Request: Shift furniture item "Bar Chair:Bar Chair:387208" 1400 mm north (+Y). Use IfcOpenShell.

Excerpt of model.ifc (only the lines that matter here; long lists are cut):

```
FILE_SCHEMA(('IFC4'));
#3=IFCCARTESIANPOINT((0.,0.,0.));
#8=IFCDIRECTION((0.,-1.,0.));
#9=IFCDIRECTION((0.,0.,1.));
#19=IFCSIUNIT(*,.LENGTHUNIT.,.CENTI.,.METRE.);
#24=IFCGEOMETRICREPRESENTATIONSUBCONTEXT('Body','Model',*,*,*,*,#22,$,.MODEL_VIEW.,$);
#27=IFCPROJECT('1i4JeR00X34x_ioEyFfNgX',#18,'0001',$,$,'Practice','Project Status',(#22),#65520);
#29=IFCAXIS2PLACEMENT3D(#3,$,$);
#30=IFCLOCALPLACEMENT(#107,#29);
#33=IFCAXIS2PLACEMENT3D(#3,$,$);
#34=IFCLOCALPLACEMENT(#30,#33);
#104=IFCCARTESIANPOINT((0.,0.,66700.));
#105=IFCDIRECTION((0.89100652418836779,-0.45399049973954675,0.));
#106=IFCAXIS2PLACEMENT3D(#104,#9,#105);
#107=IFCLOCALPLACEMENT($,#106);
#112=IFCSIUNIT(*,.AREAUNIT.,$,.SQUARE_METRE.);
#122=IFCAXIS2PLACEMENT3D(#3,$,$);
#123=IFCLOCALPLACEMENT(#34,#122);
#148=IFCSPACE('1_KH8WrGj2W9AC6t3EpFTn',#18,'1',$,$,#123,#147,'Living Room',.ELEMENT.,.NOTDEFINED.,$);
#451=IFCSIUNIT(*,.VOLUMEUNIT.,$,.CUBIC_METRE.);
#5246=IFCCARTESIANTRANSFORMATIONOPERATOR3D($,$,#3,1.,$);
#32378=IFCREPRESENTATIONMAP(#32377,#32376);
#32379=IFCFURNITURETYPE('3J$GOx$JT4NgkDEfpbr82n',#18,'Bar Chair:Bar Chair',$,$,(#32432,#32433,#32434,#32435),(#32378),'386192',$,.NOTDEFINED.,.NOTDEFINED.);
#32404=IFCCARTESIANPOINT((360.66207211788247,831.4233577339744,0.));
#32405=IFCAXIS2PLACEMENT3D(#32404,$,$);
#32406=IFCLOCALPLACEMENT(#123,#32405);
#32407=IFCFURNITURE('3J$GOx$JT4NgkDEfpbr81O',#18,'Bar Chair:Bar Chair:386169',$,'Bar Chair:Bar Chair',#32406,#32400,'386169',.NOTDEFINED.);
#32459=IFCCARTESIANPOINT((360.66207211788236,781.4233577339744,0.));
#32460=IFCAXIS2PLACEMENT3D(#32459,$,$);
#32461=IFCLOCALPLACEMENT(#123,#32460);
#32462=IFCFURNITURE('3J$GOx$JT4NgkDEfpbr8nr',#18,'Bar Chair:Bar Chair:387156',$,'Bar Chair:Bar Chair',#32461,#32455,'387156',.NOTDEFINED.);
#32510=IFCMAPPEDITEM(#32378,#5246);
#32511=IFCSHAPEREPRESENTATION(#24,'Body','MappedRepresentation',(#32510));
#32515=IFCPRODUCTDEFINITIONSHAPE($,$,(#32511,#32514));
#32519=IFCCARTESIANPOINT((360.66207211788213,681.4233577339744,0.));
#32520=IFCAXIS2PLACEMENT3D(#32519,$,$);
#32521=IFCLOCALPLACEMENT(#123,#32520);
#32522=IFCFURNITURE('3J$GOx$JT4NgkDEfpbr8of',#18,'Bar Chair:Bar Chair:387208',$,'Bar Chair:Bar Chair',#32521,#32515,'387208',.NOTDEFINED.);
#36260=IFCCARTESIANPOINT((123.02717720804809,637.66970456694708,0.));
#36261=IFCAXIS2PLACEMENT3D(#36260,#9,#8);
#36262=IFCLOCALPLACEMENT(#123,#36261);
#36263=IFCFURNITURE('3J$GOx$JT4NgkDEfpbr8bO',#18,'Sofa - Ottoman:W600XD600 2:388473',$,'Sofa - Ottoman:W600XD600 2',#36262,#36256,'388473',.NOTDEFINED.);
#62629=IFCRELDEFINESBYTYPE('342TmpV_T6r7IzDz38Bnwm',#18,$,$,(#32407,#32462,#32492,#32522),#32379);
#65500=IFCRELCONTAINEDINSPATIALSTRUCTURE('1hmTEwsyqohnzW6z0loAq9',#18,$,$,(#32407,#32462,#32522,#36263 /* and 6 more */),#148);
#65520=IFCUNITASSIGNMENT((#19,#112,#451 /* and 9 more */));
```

```python
import ifcopenshell
import ifcopenshell.api.geometry
import ifcopenshell.util.placement
import ifcopenshell.util.unit

model = ifcopenshell.open("model.ifc")
unit_scale = ifcopenshell.util.unit.calculate_unit_scale(model)

item = model.by_id(32522)
matrix = ifcopenshell.util.placement.get_local_placement(item.ObjectPlacement)
matrix[1, 3] += 1.4 / unit_scale
ifcopenshell.api.geometry.edit_object_placement(model, product=item, matrix=matrix, is_si=False)

print(ifcopenshell.util.placement.get_local_placement(item.ObjectPlacement).round(3) + 0.0)

model.write("model_edited.ifc")
```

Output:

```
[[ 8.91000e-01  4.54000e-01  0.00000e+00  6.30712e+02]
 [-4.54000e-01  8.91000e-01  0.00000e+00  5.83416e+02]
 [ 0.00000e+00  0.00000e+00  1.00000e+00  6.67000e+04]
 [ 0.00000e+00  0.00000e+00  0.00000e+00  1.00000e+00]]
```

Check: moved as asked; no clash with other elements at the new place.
